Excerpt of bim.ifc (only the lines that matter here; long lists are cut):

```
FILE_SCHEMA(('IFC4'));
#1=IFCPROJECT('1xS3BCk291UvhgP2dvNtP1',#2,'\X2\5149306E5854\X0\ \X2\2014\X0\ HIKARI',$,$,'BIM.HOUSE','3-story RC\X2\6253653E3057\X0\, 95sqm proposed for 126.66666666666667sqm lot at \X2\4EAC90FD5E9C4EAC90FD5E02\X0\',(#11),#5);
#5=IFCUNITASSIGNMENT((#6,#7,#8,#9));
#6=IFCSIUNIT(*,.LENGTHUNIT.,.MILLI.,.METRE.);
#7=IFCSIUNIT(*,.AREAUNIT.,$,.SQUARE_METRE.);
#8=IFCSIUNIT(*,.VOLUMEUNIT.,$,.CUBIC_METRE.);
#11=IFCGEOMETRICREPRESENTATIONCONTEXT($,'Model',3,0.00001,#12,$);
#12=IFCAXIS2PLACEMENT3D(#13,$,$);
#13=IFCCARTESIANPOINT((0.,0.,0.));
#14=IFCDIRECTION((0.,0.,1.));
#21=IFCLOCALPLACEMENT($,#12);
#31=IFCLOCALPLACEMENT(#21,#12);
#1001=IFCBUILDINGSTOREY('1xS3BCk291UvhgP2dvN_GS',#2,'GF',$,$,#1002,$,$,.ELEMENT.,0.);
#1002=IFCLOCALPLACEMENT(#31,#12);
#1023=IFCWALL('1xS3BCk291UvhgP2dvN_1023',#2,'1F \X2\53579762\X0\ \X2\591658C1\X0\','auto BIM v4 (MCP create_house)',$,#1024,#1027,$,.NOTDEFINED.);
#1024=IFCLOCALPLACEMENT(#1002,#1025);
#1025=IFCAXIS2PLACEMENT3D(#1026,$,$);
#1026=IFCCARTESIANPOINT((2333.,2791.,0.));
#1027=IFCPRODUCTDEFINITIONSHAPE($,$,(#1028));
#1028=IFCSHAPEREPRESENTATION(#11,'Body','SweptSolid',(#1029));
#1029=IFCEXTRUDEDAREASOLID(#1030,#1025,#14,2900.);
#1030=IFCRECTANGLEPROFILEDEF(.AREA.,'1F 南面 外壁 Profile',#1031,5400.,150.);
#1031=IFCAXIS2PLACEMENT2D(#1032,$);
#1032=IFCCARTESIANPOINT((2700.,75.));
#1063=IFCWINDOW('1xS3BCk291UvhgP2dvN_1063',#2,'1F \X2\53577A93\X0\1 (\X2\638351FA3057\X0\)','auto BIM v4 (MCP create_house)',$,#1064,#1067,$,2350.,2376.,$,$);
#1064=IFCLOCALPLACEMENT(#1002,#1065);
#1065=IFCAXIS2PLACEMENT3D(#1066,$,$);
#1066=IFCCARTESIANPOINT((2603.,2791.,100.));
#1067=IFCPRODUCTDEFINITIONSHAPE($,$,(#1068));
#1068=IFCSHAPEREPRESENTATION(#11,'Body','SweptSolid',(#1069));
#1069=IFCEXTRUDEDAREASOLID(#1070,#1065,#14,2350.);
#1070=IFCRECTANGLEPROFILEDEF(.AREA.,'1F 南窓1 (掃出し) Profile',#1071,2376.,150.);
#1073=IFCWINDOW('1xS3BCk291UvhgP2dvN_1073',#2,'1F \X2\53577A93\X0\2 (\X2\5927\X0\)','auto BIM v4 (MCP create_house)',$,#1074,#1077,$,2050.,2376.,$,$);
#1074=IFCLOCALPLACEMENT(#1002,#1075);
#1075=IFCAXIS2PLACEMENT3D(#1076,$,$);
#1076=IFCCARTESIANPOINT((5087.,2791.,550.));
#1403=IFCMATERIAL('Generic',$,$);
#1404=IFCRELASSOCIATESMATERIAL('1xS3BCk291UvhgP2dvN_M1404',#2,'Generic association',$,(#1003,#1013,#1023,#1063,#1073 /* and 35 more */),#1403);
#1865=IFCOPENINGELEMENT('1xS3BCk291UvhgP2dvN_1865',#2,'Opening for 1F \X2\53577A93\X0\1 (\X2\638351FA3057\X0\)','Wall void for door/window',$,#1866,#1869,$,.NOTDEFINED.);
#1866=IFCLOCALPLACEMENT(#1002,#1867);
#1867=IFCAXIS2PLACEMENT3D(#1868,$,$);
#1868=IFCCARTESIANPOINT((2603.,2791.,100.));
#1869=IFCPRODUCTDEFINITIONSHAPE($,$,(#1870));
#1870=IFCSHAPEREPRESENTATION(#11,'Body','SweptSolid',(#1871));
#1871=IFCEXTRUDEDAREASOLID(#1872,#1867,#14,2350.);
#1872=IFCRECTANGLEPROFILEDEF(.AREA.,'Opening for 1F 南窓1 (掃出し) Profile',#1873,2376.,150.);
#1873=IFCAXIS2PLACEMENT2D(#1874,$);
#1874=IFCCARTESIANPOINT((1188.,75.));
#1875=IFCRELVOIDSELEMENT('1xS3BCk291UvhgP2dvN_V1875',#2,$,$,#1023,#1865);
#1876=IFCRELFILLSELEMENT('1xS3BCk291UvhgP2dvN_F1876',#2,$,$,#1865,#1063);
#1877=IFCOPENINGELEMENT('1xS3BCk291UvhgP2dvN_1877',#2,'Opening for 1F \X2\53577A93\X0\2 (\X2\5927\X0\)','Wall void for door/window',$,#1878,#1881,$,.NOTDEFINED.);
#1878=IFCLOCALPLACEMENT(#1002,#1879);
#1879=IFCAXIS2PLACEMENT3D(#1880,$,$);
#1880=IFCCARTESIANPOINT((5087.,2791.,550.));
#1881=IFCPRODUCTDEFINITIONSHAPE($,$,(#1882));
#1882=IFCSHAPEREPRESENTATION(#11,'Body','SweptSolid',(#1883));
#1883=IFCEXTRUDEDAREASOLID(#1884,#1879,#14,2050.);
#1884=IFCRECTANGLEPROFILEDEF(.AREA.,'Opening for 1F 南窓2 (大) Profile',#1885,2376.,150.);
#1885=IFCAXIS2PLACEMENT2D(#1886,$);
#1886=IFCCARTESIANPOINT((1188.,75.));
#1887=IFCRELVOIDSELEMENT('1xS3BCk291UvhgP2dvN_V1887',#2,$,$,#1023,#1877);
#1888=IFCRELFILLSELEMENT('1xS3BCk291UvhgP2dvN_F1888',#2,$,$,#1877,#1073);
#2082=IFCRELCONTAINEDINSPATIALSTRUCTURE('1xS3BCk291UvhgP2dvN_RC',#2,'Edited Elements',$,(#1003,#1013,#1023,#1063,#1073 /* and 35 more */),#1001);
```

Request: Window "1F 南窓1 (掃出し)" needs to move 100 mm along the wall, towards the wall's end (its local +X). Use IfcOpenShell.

```python
import ifcopenshell
import ifcopenshell.api.geometry
import ifcopenshell.util.placement
import ifcopenshell.util.unit

model = ifcopenshell.open("bim.ifc")
unit_scale = ifcopenshell.util.unit.calculate_unit_scale(model)

window = model.by_id(1063)
opening = window.FillsVoids[0].RelatingOpeningElement
wall = opening.VoidsElements[0].RelatingBuildingElement

wall_matrix = ifcopenshell.util.placement.get_local_placement(wall.ObjectPlacement)
shift = wall_matrix[:3, 0] * 0.1 / unit_scale
before = ifcopenshell.util.placement.get_local_placement(window.ObjectPlacement)[:3, 3].copy()

# The window is not placed relative to its opening, so move both.
for product in (opening, window):
    matrix = ifcopenshell.util.placement.get_local_placement(product.ObjectPlacement)
    matrix[:3, 3] += shift
    ifcopenshell.api.geometry.edit_object_placement(model, product=product, matrix=matrix, is_si=False)

after = ifcopenshell.util.placement.get_local_placement(window.ObjectPlacement)[:3, 3]
print("window moved by", (after - before).round(3) + 0.0)

model.write("bim_edited.ifc")
```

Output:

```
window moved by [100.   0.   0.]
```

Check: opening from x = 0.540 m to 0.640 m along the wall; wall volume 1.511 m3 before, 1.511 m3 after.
